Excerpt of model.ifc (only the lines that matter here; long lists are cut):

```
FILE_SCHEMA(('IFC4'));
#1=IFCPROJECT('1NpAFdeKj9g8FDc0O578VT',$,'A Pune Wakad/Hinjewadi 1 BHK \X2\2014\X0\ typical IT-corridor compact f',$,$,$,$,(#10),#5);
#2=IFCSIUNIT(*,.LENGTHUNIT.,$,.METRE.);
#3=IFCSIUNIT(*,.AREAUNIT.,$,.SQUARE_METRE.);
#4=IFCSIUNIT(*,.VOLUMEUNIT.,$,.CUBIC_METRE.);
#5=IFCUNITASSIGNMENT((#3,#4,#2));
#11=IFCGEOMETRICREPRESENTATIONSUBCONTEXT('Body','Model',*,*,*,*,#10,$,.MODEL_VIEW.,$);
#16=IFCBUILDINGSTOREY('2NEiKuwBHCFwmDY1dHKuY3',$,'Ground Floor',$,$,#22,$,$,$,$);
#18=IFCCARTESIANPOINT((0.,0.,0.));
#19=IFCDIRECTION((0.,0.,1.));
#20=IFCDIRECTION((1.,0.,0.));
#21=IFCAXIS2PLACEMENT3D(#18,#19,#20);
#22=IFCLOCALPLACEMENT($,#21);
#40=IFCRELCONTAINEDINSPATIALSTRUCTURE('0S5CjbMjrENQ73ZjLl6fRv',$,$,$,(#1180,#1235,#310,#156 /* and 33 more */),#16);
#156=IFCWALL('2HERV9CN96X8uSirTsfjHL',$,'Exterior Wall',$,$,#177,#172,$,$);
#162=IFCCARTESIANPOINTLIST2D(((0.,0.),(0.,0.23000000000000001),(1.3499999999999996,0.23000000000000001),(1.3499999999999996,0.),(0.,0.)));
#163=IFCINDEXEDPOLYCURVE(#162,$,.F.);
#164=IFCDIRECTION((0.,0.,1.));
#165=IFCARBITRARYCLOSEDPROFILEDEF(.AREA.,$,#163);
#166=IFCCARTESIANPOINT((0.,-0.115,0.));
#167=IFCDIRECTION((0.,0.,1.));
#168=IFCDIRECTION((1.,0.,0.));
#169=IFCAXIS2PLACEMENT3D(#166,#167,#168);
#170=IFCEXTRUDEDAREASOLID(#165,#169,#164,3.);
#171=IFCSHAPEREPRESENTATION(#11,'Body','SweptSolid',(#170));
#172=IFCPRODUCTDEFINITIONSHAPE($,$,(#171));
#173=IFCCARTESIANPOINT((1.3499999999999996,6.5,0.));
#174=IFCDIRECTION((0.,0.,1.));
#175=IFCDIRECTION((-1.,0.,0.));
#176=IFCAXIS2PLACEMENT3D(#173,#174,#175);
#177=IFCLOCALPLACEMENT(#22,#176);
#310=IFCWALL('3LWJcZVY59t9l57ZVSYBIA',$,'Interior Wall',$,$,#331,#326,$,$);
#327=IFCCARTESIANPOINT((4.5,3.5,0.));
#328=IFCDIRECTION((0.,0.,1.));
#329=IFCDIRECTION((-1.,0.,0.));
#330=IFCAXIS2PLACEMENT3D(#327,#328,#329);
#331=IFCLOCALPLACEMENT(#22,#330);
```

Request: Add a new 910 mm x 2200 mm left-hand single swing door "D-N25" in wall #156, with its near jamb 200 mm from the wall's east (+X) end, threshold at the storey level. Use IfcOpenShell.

```python
import numpy as np
import ifcopenshell
import ifcopenshell.api.feature
import ifcopenshell.api.geometry
import ifcopenshell.api.root
import ifcopenshell.api.spatial
import ifcopenshell.geom
import ifcopenshell.util.element
import ifcopenshell.util.placement
import ifcopenshell.util.representation
import ifcopenshell.util.shape
import ifcopenshell.util.unit

model = ifcopenshell.open("model.ifc")
unit_scale = ifcopenshell.util.unit.calculate_unit_scale(model)
settings = ifcopenshell.geom.settings()


def volume(element):
    """Net volume in cubic metres, openings subtracted."""
    shape = ifcopenshell.geom.create_shape(settings, element)
    return ifcopenshell.util.shape.get_volume(shape.geometry)


wall = model.by_guid("2HERV9CN96X8uSirTsfjHL")
storey = ifcopenshell.util.element.get_container(wall, ifc_class="IfcBuildingStorey")
context = ifcopenshell.util.representation.get_context(model, "Model", "Body", "MODEL_VIEW")
before = volume(wall)

width, height, from_end, sill = 0.91, 2.2, 0.2, 0.0  # metres

# The wall runs along its own X axis, and the end named is its -X end.
wall_shape = ifcopenshell.geom.create_shape(settings, wall)
x, y, z = ifcopenshell.util.shape.get_vertices(wall_shape.geometry).T
start = x.min() + from_end
face, thickness = float(y.min()), float(y.max() - y.min())
wall_matrix = ifcopenshell.util.placement.get_local_placement(wall.ObjectPlacement)
level = ifcopenshell.util.placement.get_local_placement(storey.ObjectPlacement)[2, 3]


def in_wall(x, y):
    """Placement at x, y metres in the wall's axes, at sill height."""
    matrix = wall_matrix.copy()
    matrix[:, 3] = wall_matrix @ np.array([x / unit_scale, y / unit_scale, 0.0, 1.0])
    matrix[2, 3] = level + sill / unit_scale
    return matrix


# Opening: a box that overshoots both wall faces by 50 mm.
opening = ifcopenshell.api.root.create_entity(model, ifc_class="IfcOpeningElement", predefined_type="OPENING")
box = ifcopenshell.api.geometry.add_wall_representation(
    model, context=context, length=width, height=height, thickness=thickness + 0.1
)
ifcopenshell.api.geometry.assign_representation(model, product=opening, representation=box)
ifcopenshell.api.geometry.edit_object_placement(model, product=opening, matrix=in_wall(start, face - 0.05), is_si=False)
ifcopenshell.api.feature.add_feature(model, feature=opening, element=wall)

door = ifcopenshell.api.root.create_entity(model, ifc_class="IfcDoor", name="D-N25", predefined_type="DOOR")
door.OverallWidth, door.OverallHeight = width / unit_scale, height / unit_scale
door.OperationType = "SINGLE_SWING_LEFT"
body = ifcopenshell.api.geometry.add_door_representation(
    model,
    context=context,
    overall_width=door.OverallWidth,
    overall_height=door.OverallHeight,
    operation_type="SINGLE_SWING_LEFT",
    lining_properties={"LiningDepth": thickness / unit_scale, "ThresholdDepth": thickness / unit_scale},
)
ifcopenshell.api.geometry.assign_representation(model, product=door, representation=body)
ifcopenshell.api.spatial.assign_container(model, products=[door], relating_structure=storey)
ifcopenshell.api.feature.add_filling(model, opening=opening, element=door)

# The lining spans the wall, so the door starts at the wall face.
ifcopenshell.api.geometry.edit_object_placement(model, product=door, matrix=in_wall(start, face), is_si=False)

after = volume(wall)

print(f"wall volume {before:.3f} -> {after:.3f} m3")

model.write("model_v2.ifc")
```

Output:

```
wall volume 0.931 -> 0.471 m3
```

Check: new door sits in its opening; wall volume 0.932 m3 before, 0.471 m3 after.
